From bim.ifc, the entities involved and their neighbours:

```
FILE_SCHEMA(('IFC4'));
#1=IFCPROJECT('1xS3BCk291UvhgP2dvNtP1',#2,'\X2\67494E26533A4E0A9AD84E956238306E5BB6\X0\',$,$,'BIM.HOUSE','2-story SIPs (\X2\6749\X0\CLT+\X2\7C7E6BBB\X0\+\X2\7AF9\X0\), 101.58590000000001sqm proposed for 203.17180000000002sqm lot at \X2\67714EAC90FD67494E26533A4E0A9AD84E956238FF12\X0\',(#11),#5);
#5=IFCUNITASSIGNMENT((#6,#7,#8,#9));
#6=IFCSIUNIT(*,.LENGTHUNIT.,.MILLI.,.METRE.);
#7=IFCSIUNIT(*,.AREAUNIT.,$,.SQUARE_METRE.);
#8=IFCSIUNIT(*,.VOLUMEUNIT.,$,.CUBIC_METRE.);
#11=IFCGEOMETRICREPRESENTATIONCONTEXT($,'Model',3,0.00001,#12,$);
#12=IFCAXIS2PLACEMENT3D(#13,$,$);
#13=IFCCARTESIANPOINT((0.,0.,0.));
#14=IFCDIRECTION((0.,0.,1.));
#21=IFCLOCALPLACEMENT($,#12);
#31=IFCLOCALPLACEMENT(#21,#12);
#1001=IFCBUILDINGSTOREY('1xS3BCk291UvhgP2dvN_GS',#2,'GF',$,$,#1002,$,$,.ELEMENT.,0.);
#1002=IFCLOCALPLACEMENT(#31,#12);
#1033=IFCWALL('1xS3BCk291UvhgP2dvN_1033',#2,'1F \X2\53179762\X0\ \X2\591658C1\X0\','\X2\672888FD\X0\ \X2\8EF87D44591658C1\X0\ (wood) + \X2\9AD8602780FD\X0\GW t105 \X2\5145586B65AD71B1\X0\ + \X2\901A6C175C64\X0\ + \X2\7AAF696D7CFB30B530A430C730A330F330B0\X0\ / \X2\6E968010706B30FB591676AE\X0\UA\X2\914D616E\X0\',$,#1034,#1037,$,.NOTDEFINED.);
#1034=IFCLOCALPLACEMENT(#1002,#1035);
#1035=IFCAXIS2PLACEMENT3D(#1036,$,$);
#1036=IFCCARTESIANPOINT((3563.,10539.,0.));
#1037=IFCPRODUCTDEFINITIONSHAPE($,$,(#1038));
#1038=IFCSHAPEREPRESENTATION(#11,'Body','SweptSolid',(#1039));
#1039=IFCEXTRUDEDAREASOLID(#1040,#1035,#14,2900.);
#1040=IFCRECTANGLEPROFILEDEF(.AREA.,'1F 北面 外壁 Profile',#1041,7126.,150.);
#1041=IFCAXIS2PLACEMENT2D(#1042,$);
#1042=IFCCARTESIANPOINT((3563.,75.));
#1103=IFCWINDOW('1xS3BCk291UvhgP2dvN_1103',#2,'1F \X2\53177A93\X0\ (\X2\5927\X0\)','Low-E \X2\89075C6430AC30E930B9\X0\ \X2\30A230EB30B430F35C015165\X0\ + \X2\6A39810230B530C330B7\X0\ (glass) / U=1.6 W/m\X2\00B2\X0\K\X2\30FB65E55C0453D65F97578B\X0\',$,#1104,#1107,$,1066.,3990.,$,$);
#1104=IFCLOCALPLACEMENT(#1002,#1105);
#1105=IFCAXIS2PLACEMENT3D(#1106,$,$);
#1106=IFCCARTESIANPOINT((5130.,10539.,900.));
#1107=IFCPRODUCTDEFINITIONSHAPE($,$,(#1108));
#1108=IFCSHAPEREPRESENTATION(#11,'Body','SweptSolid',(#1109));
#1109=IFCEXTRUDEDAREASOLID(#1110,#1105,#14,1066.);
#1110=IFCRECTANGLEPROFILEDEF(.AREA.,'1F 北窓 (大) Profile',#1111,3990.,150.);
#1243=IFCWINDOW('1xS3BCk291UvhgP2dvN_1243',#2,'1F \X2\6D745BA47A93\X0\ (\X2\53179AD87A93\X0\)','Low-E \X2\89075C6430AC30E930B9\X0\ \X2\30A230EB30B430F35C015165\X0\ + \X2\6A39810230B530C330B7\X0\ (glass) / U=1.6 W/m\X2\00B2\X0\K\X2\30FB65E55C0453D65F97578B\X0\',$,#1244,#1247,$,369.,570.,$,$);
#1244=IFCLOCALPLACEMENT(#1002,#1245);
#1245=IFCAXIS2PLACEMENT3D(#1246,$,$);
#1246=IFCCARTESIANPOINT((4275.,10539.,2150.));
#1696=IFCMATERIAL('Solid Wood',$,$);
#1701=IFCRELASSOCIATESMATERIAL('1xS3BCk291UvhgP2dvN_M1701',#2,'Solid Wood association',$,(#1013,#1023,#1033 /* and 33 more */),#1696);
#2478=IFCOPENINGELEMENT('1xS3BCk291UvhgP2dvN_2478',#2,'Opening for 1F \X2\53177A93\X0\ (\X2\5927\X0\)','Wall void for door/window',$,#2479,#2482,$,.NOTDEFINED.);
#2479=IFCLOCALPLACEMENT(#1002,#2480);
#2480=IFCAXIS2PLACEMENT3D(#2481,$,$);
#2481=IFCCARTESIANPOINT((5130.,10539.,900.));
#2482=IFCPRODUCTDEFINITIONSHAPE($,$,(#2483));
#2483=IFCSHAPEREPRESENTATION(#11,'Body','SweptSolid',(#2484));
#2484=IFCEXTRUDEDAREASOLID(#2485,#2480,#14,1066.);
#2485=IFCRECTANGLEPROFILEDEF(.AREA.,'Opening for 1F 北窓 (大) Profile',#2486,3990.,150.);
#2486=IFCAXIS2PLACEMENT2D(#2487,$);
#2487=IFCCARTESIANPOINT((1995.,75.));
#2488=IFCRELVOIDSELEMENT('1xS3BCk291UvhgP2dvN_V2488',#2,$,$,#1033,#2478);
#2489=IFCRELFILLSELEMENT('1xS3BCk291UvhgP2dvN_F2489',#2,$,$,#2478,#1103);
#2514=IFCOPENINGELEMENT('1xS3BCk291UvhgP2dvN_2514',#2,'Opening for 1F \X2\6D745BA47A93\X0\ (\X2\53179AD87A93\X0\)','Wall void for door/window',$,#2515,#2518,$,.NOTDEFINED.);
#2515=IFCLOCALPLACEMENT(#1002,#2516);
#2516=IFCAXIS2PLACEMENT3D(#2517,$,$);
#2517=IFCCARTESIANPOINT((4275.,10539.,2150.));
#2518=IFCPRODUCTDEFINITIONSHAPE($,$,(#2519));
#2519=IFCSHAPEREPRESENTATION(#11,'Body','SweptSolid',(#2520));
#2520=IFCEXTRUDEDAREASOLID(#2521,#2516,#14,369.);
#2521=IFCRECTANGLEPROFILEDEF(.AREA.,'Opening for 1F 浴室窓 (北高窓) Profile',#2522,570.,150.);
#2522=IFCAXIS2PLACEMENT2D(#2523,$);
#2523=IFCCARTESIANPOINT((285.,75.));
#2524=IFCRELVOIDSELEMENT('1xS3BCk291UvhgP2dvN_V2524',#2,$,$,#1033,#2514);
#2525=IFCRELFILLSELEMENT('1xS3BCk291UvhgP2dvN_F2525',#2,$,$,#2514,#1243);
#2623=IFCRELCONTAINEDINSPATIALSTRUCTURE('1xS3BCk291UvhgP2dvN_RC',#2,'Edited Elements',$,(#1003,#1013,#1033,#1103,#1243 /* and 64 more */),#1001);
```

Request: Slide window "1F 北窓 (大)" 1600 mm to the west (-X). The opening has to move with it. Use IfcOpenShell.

```python
import ifcopenshell
import ifcopenshell.api.geometry
import ifcopenshell.util.placement
import ifcopenshell.util.unit

model = ifcopenshell.open("bim.ifc")
unit_scale = ifcopenshell.util.unit.calculate_unit_scale(model)

window = model.by_guid("1xS3BCk291UvhgP2dvN_1103")
opening = window.FillsVoids[0].RelatingOpeningElement
wall = opening.VoidsElements[0].RelatingBuildingElement

wall_matrix = ifcopenshell.util.placement.get_local_placement(wall.ObjectPlacement)
shift = wall_matrix[:3, 0] * -1.6 / unit_scale
before = ifcopenshell.util.placement.get_local_placement(window.ObjectPlacement)[:3, 3].copy()

# The window is not placed relative to its opening, so move both.
for product in (opening, window):
    matrix = ifcopenshell.util.placement.get_local_placement(product.ObjectPlacement)
    matrix[:3, 3] += shift
    ifcopenshell.api.geometry.edit_object_placement(model, product=product, matrix=matrix, is_si=False)

after = ifcopenshell.util.placement.get_local_placement(window.ObjectPlacement)[:3, 3]
print("window moved by", (after - before).round(3) + 0.0)

model.write("bim_edited.ifc")
```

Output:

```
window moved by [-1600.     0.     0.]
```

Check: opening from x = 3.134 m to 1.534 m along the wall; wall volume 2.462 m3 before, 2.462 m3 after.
